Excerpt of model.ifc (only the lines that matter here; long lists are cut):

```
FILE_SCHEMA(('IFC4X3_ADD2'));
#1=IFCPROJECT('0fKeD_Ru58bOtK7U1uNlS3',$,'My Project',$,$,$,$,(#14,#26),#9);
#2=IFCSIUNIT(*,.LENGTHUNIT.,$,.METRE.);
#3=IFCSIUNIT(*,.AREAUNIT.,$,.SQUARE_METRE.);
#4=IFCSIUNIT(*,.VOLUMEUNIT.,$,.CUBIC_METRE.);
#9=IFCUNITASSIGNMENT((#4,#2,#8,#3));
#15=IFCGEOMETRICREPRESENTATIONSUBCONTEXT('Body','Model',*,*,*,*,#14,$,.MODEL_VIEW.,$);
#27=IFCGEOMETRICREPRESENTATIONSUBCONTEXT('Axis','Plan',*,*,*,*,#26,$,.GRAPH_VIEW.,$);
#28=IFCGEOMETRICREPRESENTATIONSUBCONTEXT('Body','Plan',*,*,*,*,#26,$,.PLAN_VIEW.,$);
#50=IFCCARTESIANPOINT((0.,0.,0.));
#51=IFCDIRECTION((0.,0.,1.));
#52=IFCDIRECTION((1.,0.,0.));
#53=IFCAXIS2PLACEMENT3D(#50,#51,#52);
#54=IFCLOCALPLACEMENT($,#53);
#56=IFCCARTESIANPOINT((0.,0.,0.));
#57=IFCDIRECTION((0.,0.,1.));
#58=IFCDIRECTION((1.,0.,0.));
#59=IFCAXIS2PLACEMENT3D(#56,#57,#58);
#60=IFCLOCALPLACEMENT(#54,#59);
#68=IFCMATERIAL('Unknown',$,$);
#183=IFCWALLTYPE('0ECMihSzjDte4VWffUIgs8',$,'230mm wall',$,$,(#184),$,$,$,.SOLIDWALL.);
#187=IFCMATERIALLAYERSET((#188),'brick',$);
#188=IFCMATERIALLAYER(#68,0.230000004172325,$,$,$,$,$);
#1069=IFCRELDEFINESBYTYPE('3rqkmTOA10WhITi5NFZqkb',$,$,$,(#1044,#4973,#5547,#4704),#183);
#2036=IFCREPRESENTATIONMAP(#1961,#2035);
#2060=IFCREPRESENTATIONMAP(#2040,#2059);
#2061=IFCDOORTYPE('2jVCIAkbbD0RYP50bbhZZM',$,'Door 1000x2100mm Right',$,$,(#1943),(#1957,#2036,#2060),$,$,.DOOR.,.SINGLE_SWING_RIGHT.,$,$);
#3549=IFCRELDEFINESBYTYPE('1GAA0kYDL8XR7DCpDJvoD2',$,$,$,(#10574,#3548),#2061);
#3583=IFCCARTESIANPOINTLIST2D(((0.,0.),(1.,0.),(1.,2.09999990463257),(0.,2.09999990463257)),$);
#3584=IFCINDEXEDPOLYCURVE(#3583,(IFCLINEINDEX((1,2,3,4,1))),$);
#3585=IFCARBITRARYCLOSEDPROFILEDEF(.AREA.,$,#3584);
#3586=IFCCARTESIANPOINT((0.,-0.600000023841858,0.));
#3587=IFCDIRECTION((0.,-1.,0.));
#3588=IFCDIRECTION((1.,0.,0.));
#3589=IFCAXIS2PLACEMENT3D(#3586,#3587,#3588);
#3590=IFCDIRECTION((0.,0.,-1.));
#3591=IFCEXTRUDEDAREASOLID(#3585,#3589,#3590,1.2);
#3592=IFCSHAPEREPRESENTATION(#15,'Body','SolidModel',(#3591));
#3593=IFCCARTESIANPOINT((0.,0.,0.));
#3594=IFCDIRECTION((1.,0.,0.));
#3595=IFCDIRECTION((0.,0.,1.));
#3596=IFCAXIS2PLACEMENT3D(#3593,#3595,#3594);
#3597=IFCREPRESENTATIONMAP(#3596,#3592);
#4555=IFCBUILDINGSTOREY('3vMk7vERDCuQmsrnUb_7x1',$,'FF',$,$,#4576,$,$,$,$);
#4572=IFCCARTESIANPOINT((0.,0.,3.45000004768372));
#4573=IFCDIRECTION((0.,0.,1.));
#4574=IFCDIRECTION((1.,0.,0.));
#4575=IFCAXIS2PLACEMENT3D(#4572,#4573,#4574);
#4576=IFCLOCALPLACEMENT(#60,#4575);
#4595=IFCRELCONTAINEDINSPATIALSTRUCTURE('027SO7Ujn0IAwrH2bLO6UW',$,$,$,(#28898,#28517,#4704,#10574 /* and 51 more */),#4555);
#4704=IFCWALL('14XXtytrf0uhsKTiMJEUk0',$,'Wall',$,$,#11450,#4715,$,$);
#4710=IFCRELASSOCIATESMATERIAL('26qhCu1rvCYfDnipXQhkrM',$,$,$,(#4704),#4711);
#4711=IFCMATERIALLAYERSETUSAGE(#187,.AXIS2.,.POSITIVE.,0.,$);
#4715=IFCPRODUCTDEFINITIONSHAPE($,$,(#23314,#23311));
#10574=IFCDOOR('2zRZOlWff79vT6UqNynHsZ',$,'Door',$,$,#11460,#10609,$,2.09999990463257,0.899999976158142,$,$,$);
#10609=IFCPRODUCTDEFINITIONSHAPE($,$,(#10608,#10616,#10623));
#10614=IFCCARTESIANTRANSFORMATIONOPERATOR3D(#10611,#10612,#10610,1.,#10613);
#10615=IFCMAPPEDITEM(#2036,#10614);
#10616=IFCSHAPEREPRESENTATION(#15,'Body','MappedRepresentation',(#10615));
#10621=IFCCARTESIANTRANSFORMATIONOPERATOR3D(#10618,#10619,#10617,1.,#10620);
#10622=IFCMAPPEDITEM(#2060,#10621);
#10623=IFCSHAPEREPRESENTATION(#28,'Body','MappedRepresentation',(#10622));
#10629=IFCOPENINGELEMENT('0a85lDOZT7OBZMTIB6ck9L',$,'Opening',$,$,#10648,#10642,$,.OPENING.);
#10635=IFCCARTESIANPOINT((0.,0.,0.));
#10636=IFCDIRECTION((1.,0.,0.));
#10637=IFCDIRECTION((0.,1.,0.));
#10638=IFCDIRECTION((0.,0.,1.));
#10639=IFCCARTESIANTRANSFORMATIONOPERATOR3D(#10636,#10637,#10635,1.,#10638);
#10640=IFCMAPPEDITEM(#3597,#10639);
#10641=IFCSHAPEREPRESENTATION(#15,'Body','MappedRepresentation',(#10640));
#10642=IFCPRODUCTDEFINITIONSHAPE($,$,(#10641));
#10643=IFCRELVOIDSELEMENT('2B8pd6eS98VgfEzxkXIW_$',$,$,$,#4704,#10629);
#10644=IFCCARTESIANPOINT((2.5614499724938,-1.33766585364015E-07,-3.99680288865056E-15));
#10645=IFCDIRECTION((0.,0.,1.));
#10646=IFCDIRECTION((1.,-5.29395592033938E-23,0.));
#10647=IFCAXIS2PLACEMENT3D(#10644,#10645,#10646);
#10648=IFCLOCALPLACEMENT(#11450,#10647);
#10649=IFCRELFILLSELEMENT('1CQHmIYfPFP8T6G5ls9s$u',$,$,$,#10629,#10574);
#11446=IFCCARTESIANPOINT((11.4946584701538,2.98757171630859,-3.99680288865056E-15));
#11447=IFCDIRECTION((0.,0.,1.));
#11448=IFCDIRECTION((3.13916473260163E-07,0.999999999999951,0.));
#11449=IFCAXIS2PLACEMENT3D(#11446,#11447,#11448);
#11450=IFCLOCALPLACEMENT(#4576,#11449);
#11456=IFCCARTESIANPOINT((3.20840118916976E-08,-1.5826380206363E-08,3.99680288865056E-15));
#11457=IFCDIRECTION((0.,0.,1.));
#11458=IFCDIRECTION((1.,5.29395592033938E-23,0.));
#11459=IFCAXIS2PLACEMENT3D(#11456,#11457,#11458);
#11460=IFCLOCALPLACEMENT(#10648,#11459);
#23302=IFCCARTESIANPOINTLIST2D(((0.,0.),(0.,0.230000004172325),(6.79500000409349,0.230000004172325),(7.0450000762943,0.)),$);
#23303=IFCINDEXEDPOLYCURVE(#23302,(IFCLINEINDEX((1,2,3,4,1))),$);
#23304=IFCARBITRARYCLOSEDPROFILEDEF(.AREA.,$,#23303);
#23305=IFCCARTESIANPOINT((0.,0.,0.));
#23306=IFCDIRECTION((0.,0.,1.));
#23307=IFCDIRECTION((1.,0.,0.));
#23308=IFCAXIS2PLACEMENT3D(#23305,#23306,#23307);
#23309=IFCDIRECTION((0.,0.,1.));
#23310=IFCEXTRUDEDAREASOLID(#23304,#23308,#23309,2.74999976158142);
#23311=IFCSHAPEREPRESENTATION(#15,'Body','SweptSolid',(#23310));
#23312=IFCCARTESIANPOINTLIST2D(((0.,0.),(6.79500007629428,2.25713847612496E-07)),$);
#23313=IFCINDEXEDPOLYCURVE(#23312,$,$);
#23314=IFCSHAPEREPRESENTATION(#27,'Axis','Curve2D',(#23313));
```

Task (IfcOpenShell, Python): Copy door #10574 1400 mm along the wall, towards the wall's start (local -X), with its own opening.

```python
import ifcopenshell
import ifcopenshell.api.feature
import ifcopenshell.api.geometry
import ifcopenshell.api.root
import ifcopenshell.geom
import ifcopenshell.util.element
import ifcopenshell.util.placement
import ifcopenshell.util.shape
import ifcopenshell.util.unit

model = ifcopenshell.open("model.ifc")
unit_scale = ifcopenshell.util.unit.calculate_unit_scale(model)
settings = ifcopenshell.geom.settings()


def volume(element):
    """Net volume in cubic metres, openings subtracted."""
    shape = ifcopenshell.geom.create_shape(settings, element)
    return ifcopenshell.util.shape.get_volume(shape.geometry)


door = model.by_guid("2zRZOlWff79vT6UqNynHsZ")
opening = door.FillsVoids[0].RelatingOpeningElement
wall = opening.VoidsElements[0].RelatingBuildingElement
before = volume(wall)
shift = ifcopenshell.util.placement.get_local_placement(wall.ObjectPlacement)[:3, 0] * -1.4 / unit_scale

# copy_class copies the void relationship, type, container and properties, but no geometry.
new_opening = ifcopenshell.api.root.copy_class(model, product=opening)
new_opening.Representation = ifcopenshell.util.element.copy_deep(
    model, opening.Representation, exclude=["IfcGeometricRepresentationContext", "IfcRepresentationMap"]
)
new_door = ifcopenshell.api.root.copy_class(model, product=door)
new_door.Representation = ifcopenshell.util.element.copy_deep(
    model, door.Representation, exclude=["IfcGeometricRepresentationContext", "IfcRepresentationMap"]
)
ifcopenshell.api.feature.add_filling(model, opening=new_opening, element=new_door)

for old, new in ((opening, new_opening), (door, new_door)):
    matrix = ifcopenshell.util.placement.get_local_placement(old.ObjectPlacement)
    matrix[:3, 3] += shift
    ifcopenshell.api.geometry.edit_object_placement(model, product=new, matrix=matrix, is_si=False)

after = volume(wall)

print(f"wall volume {before:.3f} -> {after:.3f} m3")

model.write("model_v2.ifc")
```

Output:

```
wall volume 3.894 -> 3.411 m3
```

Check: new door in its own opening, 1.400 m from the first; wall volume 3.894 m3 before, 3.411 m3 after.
